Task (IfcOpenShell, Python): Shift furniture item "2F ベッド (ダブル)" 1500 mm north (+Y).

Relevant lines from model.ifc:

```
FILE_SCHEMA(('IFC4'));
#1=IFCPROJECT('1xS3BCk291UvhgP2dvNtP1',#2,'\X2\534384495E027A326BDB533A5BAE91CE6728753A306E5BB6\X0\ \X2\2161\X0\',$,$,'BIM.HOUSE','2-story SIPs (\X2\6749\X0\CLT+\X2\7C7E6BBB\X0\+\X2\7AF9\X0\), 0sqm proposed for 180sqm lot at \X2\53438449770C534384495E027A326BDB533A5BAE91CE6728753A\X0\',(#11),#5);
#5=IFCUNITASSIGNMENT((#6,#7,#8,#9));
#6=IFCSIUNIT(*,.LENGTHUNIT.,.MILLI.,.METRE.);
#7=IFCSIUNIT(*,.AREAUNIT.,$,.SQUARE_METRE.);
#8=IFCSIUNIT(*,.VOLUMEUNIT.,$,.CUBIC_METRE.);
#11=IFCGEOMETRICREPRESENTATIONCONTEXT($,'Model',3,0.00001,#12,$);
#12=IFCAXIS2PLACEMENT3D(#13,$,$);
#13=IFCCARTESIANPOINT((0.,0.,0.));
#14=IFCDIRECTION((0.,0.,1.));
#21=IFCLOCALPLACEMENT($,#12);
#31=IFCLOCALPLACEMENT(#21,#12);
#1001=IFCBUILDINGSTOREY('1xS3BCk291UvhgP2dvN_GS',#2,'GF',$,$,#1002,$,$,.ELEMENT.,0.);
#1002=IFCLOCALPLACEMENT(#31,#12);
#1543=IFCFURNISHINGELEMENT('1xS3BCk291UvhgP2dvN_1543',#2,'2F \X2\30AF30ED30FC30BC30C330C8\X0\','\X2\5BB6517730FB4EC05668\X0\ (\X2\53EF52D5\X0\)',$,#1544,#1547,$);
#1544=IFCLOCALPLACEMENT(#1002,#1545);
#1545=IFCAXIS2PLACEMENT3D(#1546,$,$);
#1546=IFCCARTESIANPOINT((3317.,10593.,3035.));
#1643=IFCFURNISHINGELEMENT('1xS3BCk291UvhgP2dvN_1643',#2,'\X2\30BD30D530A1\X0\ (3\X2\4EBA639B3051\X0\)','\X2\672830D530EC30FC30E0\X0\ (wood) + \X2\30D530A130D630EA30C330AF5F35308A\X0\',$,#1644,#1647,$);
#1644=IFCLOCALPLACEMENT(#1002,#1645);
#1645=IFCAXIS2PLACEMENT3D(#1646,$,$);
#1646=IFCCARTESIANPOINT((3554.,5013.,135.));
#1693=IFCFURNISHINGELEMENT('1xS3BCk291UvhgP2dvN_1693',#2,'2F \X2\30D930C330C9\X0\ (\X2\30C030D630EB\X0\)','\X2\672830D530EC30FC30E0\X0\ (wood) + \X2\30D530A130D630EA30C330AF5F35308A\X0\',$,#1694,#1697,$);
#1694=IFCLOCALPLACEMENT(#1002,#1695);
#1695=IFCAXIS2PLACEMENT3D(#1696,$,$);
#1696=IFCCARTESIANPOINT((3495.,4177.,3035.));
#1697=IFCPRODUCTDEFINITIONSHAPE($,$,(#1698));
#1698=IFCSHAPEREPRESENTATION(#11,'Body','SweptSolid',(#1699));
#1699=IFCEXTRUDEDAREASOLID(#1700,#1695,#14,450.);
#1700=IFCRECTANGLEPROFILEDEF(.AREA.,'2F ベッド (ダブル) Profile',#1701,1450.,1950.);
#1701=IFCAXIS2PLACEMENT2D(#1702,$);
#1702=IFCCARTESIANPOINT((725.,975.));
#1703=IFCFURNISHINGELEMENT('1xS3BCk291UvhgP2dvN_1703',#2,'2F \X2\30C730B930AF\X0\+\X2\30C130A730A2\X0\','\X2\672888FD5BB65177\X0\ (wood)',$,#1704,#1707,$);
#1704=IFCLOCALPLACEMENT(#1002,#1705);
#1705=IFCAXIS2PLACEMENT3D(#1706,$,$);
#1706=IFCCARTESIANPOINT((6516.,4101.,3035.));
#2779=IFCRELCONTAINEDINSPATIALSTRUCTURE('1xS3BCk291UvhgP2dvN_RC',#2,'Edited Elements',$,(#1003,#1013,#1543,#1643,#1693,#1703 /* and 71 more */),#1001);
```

```python
import ifcopenshell
import ifcopenshell.api.geometry
import ifcopenshell.util.placement
import ifcopenshell.util.unit

model = ifcopenshell.open("model.ifc")
unit_scale = ifcopenshell.util.unit.calculate_unit_scale(model)

item = model.by_guid("1xS3BCk291UvhgP2dvN_1693")
matrix = ifcopenshell.util.placement.get_local_placement(item.ObjectPlacement)
matrix[1, 3] += 1.5 / unit_scale
ifcopenshell.api.geometry.edit_object_placement(model, product=item, matrix=matrix, is_si=False)

print(ifcopenshell.util.placement.get_local_placement(item.ObjectPlacement).round(3) + 0.0)

model.write("model_updated.ifc")
```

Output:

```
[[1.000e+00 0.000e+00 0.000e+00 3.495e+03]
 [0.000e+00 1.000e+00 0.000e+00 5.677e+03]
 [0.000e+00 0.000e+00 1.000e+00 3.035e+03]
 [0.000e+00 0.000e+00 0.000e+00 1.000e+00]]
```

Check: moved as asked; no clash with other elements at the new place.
